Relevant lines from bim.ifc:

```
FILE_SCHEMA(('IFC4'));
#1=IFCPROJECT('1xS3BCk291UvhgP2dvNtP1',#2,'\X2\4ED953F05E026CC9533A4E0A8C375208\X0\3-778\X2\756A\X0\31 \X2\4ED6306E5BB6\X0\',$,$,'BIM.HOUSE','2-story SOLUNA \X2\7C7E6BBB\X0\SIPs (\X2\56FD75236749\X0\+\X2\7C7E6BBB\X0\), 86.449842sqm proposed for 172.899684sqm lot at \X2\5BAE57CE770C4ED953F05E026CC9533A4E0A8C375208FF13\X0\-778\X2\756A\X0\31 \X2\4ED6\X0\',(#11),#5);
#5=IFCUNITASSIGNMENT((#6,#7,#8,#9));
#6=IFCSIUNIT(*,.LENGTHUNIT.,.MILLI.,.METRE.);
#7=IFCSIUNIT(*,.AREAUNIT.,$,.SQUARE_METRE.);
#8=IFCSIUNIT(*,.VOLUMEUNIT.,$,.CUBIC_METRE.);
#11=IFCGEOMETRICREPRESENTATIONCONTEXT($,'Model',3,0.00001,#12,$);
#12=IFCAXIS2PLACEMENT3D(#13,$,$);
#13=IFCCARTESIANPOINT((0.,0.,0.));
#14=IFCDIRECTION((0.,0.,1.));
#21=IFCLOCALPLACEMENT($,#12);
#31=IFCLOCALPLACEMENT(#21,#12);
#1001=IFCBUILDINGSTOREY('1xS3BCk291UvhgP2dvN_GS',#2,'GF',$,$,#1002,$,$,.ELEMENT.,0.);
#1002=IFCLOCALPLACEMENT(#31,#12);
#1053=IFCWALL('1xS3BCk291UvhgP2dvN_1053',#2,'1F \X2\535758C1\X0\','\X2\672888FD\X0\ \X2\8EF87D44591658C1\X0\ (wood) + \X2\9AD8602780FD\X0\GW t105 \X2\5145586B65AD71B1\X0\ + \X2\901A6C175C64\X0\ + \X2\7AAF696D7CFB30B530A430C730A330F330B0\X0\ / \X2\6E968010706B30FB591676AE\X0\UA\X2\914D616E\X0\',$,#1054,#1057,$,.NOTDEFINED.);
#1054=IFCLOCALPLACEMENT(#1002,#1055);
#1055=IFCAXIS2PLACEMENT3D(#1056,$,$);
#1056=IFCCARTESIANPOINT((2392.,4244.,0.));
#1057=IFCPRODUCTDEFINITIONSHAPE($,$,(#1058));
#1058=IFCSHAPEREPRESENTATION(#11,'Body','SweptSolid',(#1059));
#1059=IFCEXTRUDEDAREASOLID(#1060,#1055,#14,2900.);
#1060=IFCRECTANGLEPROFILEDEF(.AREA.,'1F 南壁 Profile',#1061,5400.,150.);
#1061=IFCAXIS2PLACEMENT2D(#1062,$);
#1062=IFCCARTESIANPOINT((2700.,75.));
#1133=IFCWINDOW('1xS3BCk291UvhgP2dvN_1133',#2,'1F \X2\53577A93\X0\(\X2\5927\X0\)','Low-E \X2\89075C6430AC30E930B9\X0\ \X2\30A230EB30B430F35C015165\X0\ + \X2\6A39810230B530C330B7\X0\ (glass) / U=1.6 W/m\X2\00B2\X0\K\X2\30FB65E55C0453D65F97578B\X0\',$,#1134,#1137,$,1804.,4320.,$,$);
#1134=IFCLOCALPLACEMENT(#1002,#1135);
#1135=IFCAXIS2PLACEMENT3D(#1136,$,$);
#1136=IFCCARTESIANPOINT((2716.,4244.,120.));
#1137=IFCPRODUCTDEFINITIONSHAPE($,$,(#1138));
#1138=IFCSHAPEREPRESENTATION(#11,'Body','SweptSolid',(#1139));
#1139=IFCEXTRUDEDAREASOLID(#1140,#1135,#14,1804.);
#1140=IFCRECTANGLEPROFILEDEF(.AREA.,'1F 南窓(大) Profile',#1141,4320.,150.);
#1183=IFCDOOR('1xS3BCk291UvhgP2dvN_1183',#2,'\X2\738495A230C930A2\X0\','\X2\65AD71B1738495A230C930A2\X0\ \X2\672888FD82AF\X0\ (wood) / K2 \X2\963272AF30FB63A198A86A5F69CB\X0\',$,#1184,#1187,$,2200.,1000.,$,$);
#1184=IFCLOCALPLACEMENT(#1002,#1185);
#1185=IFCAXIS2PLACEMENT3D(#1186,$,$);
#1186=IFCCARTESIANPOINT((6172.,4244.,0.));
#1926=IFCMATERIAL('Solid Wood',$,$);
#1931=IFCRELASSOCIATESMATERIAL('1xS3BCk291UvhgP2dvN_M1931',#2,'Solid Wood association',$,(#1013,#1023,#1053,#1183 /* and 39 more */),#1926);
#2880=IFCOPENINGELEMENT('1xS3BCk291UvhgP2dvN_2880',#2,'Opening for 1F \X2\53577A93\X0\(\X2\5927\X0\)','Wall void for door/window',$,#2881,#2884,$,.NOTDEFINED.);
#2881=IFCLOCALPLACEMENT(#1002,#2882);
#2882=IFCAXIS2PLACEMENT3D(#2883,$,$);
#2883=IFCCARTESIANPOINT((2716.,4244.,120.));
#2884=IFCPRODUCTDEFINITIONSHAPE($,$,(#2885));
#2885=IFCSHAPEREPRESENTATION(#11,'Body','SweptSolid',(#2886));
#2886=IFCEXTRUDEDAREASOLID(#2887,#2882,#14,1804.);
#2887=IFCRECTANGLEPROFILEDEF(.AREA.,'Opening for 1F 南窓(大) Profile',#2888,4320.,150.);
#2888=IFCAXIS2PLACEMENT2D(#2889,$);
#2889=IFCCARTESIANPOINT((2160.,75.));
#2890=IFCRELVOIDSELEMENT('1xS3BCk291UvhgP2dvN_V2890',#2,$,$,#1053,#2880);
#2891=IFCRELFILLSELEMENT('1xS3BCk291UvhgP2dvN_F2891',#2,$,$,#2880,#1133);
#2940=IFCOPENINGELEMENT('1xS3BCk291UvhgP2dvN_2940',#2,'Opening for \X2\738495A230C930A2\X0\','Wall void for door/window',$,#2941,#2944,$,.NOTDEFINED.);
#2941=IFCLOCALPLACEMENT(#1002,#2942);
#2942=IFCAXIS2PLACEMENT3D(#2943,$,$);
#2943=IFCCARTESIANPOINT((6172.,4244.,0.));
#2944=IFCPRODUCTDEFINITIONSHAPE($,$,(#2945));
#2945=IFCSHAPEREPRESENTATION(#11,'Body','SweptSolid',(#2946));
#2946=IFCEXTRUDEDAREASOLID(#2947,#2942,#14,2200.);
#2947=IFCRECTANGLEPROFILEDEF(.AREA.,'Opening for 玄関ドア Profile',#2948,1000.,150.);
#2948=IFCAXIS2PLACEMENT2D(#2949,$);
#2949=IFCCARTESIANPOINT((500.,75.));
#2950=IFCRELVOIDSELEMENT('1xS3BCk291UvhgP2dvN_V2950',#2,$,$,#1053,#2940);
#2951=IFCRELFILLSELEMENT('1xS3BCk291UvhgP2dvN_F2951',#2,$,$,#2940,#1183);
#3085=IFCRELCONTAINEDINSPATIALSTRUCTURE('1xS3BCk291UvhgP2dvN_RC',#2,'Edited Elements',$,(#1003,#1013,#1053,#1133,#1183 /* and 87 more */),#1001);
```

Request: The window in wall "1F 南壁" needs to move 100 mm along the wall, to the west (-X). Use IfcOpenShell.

```python
import ifcopenshell
import ifcopenshell.api.geometry
import ifcopenshell.util.placement
import ifcopenshell.util.unit

model = ifcopenshell.open("bim.ifc")
unit_scale = ifcopenshell.util.unit.calculate_unit_scale(model)

window = model.by_id(1133)
opening = window.FillsVoids[0].RelatingOpeningElement
wall = opening.VoidsElements[0].RelatingBuildingElement

wall_matrix = ifcopenshell.util.placement.get_local_placement(wall.ObjectPlacement)
shift = wall_matrix[:3, 0] * -0.1 / unit_scale
before = ifcopenshell.util.placement.get_local_placement(window.ObjectPlacement)[:3, 3].copy()

# The window is not placed relative to its opening, so move both.
for product in (opening, window):
    matrix = ifcopenshell.util.placement.get_local_placement(product.ObjectPlacement)
    matrix[:3, 3] += shift
    ifcopenshell.api.geometry.edit_object_placement(model, product=product, matrix=matrix, is_si=False)

after = ifcopenshell.util.placement.get_local_placement(window.ObjectPlacement)[:3, 3]
print("window moved by", (after - before).round(3) + 0.0)

model.write("bim_v2.ifc")
```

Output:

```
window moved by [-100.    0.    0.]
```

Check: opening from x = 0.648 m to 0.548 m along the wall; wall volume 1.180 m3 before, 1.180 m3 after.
